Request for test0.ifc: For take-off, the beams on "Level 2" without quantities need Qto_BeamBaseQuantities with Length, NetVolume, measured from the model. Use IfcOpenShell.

First a look at what the model holds.

```python
import ifcopenshell
import ifcopenshell.util.element
import ifcopenshell.util.unit

model = ifcopenshell.open("test0.ifc")
print(model.schema)
for unit_type in ("LENGTHUNIT", "AREAUNIT", "VOLUMEUNIT"):
    print(unit_type, ifcopenshell.util.unit.calculate_unit_scale(model, unit_type))
storey = next(s for s in model.by_type("IfcBuildingStorey") if s.Name == "Level 2")
beams = [e for e in ifcopenshell.util.element.get_decomposition(storey) if e.is_a("IfcBeam")]
for e in sorted(beams, key=lambda e: e.id()):
    print(e.id(), e.is_a(), e.Name, list(ifcopenshell.util.element.get_psets(e, qtos_only=True)), sep=" | ")
```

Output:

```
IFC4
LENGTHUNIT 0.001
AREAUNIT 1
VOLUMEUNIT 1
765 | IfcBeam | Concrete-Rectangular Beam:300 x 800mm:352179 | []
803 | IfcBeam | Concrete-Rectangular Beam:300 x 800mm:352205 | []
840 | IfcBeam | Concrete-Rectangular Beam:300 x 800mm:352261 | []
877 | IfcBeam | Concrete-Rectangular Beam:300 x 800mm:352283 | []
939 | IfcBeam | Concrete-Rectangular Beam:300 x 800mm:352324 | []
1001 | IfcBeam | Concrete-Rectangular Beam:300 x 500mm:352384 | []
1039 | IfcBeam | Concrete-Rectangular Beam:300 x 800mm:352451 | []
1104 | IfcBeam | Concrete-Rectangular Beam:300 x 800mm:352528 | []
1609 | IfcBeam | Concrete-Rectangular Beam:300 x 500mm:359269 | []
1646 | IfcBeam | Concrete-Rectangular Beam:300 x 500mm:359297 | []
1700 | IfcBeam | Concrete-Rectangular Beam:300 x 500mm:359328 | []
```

```python
import ifcopenshell
import ifcopenshell.api.pset
import ifcopenshell.geom
import ifcopenshell.util.element
import ifcopenshell.util.shape
import ifcopenshell.util.unit

model = ifcopenshell.open("test0.ifc")
unit_scale = ifcopenshell.util.unit.calculate_unit_scale(model)
volume_scale = ifcopenshell.util.unit.calculate_unit_scale(model, "VOLUMEUNIT")
settings = ifcopenshell.geom.settings()

storey = next(s for s in model.by_type("IfcBuildingStorey") if s.Name == "Level 2")
beams = [e for e in ifcopenshell.util.element.get_decomposition(storey) if e.is_a("IfcBeam")]

for e in sorted(beams, key=lambda e: e.id()):
    if ifcopenshell.util.element.get_psets(e, qtos_only=True, should_inherit=False):
        continue
    # Geometry comes back in metres, in the element's own axes.
    shape = ifcopenshell.geom.create_shape(settings, e)
    values = {
        "Length": ifcopenshell.util.shape.get_max_xyz(shape.geometry) / unit_scale,
        "NetVolume": ifcopenshell.util.shape.get_volume(shape.geometry) / volume_scale,
    }
    qto = ifcopenshell.api.pset.add_qto(model, product=e, name="Qto_BeamBaseQuantities")
    ifcopenshell.api.pset.edit_qto(model, qto=qto, properties=values)
    print(e.id(), {k: round(v, 3) for k, v in values.items()})

model.write("test0_edited.ifc")
```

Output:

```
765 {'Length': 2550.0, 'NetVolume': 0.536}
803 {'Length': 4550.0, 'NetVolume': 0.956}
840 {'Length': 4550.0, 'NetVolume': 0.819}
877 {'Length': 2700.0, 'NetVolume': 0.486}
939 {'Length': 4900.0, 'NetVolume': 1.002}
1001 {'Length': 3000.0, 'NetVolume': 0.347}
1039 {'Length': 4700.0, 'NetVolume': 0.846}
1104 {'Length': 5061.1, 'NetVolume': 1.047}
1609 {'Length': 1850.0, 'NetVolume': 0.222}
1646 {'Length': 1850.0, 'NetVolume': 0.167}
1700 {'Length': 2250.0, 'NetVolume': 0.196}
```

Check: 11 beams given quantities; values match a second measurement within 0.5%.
